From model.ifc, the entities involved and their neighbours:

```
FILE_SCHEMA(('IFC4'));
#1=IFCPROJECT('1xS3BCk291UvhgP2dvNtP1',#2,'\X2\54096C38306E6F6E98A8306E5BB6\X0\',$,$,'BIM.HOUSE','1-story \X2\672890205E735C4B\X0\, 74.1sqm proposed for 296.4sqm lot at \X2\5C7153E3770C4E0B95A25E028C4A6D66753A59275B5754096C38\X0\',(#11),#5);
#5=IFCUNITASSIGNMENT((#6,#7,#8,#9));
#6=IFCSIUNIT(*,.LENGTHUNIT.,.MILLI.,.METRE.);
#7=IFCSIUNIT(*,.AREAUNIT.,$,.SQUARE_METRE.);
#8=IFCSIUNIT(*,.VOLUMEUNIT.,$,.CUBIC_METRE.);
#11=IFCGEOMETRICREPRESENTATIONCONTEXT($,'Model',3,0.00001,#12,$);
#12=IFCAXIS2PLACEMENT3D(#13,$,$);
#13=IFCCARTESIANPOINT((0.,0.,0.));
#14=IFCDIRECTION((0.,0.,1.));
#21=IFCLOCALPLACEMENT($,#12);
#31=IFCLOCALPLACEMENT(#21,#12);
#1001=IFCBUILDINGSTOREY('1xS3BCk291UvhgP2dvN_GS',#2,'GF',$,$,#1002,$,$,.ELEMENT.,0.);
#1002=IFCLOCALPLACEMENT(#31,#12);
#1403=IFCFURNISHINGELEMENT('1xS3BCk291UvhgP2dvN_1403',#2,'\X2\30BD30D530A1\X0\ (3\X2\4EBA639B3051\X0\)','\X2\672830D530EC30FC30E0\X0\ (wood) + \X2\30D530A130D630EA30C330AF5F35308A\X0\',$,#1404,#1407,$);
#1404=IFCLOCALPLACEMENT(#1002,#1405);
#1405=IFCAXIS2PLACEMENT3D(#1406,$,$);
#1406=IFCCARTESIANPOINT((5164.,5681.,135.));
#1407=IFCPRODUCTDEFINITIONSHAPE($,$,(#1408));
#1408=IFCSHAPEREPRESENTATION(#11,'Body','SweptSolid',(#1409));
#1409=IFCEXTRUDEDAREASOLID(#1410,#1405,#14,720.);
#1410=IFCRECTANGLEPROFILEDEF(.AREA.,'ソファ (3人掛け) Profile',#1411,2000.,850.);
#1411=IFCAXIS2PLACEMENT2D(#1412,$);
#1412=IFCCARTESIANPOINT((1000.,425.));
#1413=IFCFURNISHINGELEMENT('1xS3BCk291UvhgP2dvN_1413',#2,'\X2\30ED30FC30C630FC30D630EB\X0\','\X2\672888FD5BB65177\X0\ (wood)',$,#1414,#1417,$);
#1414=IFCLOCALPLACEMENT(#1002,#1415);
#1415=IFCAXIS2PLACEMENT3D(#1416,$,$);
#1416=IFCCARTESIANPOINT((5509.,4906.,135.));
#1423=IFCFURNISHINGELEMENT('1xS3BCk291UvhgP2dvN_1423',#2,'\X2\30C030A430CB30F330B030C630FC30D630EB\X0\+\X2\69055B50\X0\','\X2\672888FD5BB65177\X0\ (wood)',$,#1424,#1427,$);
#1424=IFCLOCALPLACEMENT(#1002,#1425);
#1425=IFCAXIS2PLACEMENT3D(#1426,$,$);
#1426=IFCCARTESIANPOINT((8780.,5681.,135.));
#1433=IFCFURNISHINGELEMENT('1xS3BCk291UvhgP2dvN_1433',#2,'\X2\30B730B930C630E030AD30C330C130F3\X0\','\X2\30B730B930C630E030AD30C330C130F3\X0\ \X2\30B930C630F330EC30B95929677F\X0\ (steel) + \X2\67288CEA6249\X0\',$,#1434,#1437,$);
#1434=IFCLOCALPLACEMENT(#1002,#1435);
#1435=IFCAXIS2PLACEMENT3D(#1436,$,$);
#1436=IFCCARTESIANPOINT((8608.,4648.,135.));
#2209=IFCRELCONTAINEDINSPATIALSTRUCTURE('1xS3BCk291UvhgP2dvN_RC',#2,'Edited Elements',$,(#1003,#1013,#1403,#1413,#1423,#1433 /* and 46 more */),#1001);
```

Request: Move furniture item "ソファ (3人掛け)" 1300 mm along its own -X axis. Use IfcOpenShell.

```python
import ifcopenshell
import ifcopenshell.api.geometry
import ifcopenshell.util.placement

model = ifcopenshell.open("model.ifc")

item = model.by_id(1403)
matrix = ifcopenshell.util.placement.get_local_placement(item.ObjectPlacement)
matrix[:3, 3] -= matrix[:3, 0] * 1300.0
ifcopenshell.api.geometry.edit_object_placement(model, product=item, matrix=matrix, is_si=False)

print(ifcopenshell.util.placement.get_local_placement(item.ObjectPlacement).round(3) + 0.0)

model.write("model_rev.ifc")
```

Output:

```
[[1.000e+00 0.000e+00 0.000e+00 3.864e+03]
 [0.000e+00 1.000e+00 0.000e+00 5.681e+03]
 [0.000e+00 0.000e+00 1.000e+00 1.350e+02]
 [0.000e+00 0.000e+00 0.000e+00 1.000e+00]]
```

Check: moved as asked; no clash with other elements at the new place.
